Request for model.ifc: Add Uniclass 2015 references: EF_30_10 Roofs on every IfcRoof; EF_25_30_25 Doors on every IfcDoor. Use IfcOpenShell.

First a look at what the model holds.

```python
import ifcopenshell

model = ifcopenshell.open("model.ifc")
print(model.schema)
print("classifications:", [c.Name for c in model.by_type("IfcClassification")])
for ifc_class in ("IfcDoor", "IfcRoof", "IfcStair", "IfcWall", "IfcWindow"):
    print(ifc_class, len(model.by_type(ifc_class)))
```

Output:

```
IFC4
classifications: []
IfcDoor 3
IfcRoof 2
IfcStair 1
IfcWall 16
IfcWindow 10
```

```python
import ifcopenshell
import ifcopenshell.api.classification

model = ifcopenshell.open("model.ifc")

system = ifcopenshell.api.classification.add_classification(model, classification="Uniclass 2015")

codes = {
    "IfcRoof": ("EF_30_10", "Roofs"),
    "IfcDoor": ("EF_25_30_25", "Doors"),
}
for ifc_class, (code, name) in codes.items():
    products = model.by_type(ifc_class)
    ifcopenshell.api.classification.add_reference(
        model, products=products, classification=system, identification=code, name=name
    )
    print(code, len(products))

model.write("model_edited.ifc")
```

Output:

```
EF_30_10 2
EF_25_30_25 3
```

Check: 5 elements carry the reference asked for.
